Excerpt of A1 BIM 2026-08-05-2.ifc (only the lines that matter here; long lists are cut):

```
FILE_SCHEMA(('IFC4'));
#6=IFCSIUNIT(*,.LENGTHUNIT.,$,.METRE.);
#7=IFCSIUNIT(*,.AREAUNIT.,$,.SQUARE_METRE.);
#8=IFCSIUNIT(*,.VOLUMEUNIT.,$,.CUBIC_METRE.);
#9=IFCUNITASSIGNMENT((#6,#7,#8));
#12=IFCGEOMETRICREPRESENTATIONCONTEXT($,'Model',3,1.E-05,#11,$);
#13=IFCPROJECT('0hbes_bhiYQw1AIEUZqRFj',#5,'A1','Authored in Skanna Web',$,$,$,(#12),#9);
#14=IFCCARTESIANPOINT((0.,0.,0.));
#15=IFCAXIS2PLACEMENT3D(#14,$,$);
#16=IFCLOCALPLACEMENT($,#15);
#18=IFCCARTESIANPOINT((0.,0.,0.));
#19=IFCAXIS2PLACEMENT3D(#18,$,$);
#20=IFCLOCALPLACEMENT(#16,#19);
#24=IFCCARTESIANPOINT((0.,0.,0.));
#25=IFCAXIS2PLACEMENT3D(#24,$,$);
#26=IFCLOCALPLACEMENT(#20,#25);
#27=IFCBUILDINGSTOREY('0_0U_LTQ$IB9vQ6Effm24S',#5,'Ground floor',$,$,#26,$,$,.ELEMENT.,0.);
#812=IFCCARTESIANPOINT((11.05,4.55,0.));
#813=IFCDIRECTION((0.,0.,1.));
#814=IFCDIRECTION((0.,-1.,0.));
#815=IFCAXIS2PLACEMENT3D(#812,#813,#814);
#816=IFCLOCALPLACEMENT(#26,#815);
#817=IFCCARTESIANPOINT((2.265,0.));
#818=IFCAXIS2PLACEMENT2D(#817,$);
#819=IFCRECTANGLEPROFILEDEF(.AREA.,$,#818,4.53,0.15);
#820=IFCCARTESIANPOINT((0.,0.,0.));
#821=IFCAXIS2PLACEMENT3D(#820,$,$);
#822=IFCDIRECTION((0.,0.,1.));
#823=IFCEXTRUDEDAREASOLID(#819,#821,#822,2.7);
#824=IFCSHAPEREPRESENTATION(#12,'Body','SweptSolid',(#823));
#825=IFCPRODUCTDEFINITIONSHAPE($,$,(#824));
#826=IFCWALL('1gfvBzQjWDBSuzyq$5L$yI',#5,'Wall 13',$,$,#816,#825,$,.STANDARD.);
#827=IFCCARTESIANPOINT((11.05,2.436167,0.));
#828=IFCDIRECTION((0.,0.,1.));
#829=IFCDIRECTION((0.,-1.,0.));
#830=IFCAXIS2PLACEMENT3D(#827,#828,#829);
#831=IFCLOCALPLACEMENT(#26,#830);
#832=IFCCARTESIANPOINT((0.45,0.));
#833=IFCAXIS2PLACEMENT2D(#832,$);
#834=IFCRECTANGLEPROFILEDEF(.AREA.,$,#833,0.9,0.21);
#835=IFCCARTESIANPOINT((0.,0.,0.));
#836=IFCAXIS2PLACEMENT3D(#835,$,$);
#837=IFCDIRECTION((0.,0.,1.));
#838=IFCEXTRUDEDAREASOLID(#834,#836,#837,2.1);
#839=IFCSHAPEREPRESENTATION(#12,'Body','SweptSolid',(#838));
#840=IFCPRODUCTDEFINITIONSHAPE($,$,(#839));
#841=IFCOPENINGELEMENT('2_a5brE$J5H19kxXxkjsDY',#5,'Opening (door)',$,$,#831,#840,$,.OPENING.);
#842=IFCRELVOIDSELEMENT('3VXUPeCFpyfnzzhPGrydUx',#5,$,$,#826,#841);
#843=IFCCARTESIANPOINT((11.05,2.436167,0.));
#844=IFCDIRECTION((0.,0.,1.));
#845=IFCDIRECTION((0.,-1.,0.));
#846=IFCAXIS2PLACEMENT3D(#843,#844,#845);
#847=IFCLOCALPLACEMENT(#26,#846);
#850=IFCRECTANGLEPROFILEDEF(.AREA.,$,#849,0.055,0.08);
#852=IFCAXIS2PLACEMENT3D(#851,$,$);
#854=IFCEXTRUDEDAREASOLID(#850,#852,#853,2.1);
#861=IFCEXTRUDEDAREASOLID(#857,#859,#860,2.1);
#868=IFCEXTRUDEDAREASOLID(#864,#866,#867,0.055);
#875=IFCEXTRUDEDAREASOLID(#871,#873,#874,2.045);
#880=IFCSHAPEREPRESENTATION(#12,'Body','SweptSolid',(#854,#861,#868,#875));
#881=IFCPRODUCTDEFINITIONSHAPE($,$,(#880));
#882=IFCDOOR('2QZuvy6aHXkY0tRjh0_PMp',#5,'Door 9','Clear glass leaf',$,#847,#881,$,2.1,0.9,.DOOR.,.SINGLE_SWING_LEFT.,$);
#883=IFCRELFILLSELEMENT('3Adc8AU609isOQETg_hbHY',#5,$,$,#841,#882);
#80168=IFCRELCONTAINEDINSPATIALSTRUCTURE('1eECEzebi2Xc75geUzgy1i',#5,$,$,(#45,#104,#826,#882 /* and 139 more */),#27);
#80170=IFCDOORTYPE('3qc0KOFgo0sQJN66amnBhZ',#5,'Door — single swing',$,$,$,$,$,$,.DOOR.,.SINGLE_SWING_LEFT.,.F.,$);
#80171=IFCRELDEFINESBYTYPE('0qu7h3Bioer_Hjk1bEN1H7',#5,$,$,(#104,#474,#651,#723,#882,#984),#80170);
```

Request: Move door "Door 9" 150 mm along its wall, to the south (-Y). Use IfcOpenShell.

```python
import ifcopenshell
import ifcopenshell.api.geometry
import ifcopenshell.util.placement
import ifcopenshell.util.unit

model = ifcopenshell.open("A1 BIM 2026-08-05-2.ifc")
unit_scale = ifcopenshell.util.unit.calculate_unit_scale(model)

door = model.by_id(882)
opening = door.FillsVoids[0].RelatingOpeningElement
wall = opening.VoidsElements[0].RelatingBuildingElement

wall_matrix = ifcopenshell.util.placement.get_local_placement(wall.ObjectPlacement)
shift = wall_matrix[:3, 0] * 0.15 / unit_scale
before = ifcopenshell.util.placement.get_local_placement(door.ObjectPlacement)[:3, 3].copy()

# The door is not placed relative to its opening, so move both.
for product in (opening, door):
    matrix = ifcopenshell.util.placement.get_local_placement(product.ObjectPlacement)
    matrix[:3, 3] += shift
    ifcopenshell.api.geometry.edit_object_placement(model, product=product, matrix=matrix, is_si=False)

after = ifcopenshell.util.placement.get_local_placement(door.ObjectPlacement)[:3, 3]
print("door moved by", (after - before).round(3) + 0.0)

model.write("A1 BIM 2026-08-05-2_edited.ifc")
```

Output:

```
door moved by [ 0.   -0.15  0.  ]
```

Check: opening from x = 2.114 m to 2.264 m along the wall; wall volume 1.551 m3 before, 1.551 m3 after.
